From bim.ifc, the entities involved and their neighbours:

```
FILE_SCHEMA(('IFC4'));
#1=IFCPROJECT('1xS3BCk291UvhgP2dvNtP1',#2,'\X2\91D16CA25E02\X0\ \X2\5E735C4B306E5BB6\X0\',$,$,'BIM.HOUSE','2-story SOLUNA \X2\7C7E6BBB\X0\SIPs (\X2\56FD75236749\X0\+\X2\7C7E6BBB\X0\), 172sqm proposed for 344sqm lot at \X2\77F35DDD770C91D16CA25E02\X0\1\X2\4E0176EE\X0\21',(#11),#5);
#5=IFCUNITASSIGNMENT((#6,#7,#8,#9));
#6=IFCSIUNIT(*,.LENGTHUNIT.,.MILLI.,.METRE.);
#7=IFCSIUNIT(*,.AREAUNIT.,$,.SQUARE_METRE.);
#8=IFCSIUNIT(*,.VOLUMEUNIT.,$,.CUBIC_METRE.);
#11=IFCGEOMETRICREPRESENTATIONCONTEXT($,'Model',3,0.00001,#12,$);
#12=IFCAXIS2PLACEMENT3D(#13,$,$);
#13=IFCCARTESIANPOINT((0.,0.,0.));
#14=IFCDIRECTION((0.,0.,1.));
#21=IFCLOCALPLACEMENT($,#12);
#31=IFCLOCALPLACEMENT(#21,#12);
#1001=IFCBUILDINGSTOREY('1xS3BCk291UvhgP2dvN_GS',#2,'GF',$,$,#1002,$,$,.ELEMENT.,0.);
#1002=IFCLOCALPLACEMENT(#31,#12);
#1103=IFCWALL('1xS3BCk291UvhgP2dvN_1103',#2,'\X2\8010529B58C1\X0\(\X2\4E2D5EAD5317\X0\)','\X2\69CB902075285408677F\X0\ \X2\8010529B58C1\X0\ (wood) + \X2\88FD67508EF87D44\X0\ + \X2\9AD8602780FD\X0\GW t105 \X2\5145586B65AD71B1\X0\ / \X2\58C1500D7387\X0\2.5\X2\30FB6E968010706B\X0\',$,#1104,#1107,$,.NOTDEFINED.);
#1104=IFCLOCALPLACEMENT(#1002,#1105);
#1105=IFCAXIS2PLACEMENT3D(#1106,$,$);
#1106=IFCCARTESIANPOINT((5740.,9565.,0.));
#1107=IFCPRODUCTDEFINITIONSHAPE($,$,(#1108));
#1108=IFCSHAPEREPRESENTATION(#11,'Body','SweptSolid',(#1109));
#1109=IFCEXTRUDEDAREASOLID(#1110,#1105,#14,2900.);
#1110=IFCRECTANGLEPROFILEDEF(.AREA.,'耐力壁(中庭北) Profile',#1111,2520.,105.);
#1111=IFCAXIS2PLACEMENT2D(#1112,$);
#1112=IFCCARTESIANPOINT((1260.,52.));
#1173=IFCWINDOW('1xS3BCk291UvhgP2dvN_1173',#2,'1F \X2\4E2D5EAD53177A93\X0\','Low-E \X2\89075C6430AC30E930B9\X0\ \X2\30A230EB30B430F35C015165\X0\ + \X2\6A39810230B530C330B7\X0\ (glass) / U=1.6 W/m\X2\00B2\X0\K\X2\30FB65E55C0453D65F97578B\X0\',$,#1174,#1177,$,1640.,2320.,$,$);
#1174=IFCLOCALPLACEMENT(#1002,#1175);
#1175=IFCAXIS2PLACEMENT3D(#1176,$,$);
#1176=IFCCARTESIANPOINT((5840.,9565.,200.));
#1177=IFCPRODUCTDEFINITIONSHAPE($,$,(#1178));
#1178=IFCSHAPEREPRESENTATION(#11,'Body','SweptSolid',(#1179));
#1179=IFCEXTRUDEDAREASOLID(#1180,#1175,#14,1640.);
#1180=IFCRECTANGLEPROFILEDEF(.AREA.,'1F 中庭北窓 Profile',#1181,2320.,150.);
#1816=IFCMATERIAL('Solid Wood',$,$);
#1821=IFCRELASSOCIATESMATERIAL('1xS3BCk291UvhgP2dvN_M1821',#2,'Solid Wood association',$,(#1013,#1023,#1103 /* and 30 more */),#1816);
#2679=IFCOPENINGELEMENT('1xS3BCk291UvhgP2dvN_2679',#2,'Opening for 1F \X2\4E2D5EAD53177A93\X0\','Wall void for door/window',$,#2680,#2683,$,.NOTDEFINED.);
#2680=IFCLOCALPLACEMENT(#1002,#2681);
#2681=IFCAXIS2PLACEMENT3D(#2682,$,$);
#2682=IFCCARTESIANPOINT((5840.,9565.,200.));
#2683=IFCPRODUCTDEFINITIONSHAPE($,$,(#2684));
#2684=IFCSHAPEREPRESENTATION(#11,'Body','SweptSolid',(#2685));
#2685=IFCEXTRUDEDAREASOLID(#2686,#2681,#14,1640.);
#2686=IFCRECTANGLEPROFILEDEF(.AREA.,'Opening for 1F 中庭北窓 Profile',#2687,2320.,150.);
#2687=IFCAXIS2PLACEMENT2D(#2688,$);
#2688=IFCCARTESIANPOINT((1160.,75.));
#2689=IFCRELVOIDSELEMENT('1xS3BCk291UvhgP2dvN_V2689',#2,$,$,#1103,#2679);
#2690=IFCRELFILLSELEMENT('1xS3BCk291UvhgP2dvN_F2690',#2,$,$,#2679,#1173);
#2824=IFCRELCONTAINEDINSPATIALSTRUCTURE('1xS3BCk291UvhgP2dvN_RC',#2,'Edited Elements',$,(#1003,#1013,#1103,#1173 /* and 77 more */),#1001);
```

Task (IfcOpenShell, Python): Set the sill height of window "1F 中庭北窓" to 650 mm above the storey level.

```python
import numpy as np
import ifcopenshell
import ifcopenshell.api.geometry
import ifcopenshell.geom
import ifcopenshell.util.element
import ifcopenshell.util.placement
import ifcopenshell.util.shape
import ifcopenshell.util.unit

model = ifcopenshell.open("bim.ifc")
unit_scale = ifcopenshell.util.unit.calculate_unit_scale(model)

window = model.by_id(1173)
opening = window.FillsVoids[0].RelatingOpeningElement
storey = ifcopenshell.util.element.get_container(window, ifc_class="IfcBuildingStorey")
level = ifcopenshell.util.placement.get_local_placement(storey.ObjectPlacement)[2, 3]

# The opening's origin need not be at the sill, so measure its lowest point.
shape = ifcopenshell.geom.create_shape(ifcopenshell.geom.settings(), opening)
bottom = ifcopenshell.util.shape.get_shape_bottom_elevation(shape, shape.geometry) / unit_scale
dz = level + 650.0 - bottom

shift = np.array([0.0, 0.0, dz])
# The window is not placed relative to its opening, so move both.
for product in (opening, window):
    matrix = ifcopenshell.util.placement.get_local_placement(product.ObjectPlacement)
    matrix[:3, 3] += shift
    ifcopenshell.api.geometry.edit_object_placement(model, product=product, matrix=matrix, is_si=False)

print(f"moved by {dz * unit_scale:+.3f} m")

model.write("bim_v2.ifc")
```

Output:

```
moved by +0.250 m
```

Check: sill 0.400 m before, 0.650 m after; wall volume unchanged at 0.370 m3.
